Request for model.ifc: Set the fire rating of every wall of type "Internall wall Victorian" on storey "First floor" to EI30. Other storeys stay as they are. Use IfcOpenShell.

First a look at what the model holds.

```python
import ifcopenshell
import ifcopenshell.util.element

model = ifcopenshell.open("model.ifc")
print(model.schema)
storey = next(s for s in model.by_type("IfcBuildingStorey") if s.Name == "First floor")
walls = [e for e in ifcopenshell.util.element.get_decomposition(storey) if e.is_a("IfcWall")]
seen = {}
for e in walls:
    element_type = ifcopenshell.util.element.get_type(e)
    key = (element_type.Name if element_type != e and element_type else None, ifcopenshell.util.element.get_pset(e, "Pset_WallCommon", "FireRating"))
    seen[key] = seen.get(key, 0) + 1
for (name, value), count in sorted(seen.items(), key=str):
    print(count, "x", name, "|", value)
```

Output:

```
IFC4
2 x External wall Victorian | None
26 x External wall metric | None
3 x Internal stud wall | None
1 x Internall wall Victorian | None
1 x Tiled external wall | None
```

```python
import ifcopenshell
import ifcopenshell.api.pset
import ifcopenshell.util.element

model = ifcopenshell.open("model.ifc")

storey = next(s for s in model.by_type("IfcBuildingStorey") if s.Name == "First floor")
walls = [e for e in ifcopenshell.util.element.get_decomposition(storey) if e.is_a("IfcWall")]

count = 0
for e in walls:
    element_type = ifcopenshell.util.element.get_type(e)
    if element_type in (None, e) or element_type.Name != "Internall wall Victorian":
        continue
    # add_pset returns the element's existing set when there is one.
    pset = ifcopenshell.api.pset.add_pset(model, product=e, name="Pset_WallCommon")
    ifcopenshell.api.pset.edit_pset(model, pset=pset, properties={"FireRating": "EI30"})
    count += 1

print(count, "walls updated")

model.write("model-out.ifc")
```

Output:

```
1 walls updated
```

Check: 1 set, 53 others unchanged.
